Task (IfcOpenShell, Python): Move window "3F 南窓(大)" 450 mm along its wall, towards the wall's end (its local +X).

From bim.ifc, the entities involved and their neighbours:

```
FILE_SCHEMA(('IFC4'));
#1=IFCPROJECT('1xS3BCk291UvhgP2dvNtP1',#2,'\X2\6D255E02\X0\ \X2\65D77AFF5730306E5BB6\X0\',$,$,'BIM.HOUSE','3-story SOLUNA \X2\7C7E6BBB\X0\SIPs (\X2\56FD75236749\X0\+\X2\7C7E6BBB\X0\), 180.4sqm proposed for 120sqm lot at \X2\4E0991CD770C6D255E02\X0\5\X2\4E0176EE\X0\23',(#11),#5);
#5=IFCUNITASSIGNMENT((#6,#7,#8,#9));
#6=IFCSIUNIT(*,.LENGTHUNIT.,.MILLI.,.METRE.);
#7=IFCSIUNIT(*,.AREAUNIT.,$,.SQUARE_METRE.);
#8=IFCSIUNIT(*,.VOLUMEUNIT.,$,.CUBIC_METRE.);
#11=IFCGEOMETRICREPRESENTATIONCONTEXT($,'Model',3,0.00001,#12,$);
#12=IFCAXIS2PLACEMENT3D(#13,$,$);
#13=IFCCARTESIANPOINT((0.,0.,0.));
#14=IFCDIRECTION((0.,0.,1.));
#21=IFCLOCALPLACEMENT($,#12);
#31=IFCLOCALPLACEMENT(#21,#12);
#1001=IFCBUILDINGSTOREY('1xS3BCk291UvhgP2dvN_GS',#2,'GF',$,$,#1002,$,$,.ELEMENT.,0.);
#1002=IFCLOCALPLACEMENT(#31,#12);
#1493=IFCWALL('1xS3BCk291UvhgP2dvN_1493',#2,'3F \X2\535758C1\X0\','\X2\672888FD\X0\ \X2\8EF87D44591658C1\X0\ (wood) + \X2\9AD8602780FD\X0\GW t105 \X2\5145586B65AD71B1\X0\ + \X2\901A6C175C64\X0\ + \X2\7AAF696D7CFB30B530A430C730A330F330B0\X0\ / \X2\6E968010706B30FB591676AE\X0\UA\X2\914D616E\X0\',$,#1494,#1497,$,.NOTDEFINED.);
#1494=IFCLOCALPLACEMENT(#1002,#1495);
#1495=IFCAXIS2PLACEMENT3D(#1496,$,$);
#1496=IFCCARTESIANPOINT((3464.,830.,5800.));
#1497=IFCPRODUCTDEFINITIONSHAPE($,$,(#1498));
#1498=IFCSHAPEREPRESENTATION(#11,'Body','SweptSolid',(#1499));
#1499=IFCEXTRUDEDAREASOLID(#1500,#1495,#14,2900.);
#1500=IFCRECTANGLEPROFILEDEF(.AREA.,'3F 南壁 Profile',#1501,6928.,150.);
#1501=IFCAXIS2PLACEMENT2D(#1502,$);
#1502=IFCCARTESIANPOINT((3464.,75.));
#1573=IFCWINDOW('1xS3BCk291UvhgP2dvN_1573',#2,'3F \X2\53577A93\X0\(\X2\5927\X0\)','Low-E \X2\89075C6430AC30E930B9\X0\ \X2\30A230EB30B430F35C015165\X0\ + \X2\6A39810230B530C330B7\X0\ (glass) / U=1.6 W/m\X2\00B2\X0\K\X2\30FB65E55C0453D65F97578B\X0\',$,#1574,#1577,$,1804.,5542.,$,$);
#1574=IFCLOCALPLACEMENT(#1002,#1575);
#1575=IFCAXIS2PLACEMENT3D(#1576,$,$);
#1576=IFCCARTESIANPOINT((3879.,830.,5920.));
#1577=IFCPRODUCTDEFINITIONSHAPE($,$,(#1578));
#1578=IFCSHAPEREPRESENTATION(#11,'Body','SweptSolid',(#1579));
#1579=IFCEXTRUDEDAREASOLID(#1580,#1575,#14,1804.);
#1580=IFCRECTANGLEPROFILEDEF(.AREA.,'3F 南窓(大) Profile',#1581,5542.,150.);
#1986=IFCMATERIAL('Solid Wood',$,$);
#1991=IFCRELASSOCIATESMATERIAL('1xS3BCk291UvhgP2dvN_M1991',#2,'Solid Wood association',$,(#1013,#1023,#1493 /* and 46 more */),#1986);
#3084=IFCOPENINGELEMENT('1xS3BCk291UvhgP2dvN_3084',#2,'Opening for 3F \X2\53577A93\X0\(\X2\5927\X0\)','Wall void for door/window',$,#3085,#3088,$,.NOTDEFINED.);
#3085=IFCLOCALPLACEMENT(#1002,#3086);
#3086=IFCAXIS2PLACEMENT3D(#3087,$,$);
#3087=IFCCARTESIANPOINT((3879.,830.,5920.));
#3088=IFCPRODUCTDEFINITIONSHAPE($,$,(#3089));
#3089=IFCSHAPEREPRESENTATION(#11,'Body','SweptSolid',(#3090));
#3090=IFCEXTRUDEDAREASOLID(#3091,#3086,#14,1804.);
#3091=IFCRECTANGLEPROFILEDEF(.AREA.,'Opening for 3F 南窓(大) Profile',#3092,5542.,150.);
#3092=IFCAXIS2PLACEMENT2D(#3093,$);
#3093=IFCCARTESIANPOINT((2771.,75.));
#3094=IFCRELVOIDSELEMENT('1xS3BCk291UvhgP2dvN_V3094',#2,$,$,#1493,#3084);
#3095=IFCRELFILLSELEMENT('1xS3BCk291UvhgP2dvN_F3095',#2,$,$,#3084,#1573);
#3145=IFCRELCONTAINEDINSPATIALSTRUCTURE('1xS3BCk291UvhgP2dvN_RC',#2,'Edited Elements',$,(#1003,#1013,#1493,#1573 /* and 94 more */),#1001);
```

```python
import ifcopenshell
import ifcopenshell.api.geometry
import ifcopenshell.util.placement

model = ifcopenshell.open("bim.ifc")

window = model.by_guid("1xS3BCk291UvhgP2dvN_1573")
opening = window.FillsVoids[0].RelatingOpeningElement
wall = opening.VoidsElements[0].RelatingBuildingElement

wall_matrix = ifcopenshell.util.placement.get_local_placement(wall.ObjectPlacement)
shift = wall_matrix[:3, 0] * 450.0
before = ifcopenshell.util.placement.get_local_placement(window.ObjectPlacement)[:3, 3].copy()

# The window is not placed relative to its opening, so move both.
for product in (opening, window):
    matrix = ifcopenshell.util.placement.get_local_placement(product.ObjectPlacement)
    matrix[:3, 3] += shift
    ifcopenshell.api.geometry.edit_object_placement(model, product=product, matrix=matrix, is_si=False)

after = ifcopenshell.util.placement.get_local_placement(window.ObjectPlacement)[:3, 3]
print("window moved by", (after - before).round(3) + 0.0)

model.write("bim-out.ifc")
```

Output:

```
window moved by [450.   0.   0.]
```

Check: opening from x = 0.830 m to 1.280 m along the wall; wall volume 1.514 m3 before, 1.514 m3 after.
